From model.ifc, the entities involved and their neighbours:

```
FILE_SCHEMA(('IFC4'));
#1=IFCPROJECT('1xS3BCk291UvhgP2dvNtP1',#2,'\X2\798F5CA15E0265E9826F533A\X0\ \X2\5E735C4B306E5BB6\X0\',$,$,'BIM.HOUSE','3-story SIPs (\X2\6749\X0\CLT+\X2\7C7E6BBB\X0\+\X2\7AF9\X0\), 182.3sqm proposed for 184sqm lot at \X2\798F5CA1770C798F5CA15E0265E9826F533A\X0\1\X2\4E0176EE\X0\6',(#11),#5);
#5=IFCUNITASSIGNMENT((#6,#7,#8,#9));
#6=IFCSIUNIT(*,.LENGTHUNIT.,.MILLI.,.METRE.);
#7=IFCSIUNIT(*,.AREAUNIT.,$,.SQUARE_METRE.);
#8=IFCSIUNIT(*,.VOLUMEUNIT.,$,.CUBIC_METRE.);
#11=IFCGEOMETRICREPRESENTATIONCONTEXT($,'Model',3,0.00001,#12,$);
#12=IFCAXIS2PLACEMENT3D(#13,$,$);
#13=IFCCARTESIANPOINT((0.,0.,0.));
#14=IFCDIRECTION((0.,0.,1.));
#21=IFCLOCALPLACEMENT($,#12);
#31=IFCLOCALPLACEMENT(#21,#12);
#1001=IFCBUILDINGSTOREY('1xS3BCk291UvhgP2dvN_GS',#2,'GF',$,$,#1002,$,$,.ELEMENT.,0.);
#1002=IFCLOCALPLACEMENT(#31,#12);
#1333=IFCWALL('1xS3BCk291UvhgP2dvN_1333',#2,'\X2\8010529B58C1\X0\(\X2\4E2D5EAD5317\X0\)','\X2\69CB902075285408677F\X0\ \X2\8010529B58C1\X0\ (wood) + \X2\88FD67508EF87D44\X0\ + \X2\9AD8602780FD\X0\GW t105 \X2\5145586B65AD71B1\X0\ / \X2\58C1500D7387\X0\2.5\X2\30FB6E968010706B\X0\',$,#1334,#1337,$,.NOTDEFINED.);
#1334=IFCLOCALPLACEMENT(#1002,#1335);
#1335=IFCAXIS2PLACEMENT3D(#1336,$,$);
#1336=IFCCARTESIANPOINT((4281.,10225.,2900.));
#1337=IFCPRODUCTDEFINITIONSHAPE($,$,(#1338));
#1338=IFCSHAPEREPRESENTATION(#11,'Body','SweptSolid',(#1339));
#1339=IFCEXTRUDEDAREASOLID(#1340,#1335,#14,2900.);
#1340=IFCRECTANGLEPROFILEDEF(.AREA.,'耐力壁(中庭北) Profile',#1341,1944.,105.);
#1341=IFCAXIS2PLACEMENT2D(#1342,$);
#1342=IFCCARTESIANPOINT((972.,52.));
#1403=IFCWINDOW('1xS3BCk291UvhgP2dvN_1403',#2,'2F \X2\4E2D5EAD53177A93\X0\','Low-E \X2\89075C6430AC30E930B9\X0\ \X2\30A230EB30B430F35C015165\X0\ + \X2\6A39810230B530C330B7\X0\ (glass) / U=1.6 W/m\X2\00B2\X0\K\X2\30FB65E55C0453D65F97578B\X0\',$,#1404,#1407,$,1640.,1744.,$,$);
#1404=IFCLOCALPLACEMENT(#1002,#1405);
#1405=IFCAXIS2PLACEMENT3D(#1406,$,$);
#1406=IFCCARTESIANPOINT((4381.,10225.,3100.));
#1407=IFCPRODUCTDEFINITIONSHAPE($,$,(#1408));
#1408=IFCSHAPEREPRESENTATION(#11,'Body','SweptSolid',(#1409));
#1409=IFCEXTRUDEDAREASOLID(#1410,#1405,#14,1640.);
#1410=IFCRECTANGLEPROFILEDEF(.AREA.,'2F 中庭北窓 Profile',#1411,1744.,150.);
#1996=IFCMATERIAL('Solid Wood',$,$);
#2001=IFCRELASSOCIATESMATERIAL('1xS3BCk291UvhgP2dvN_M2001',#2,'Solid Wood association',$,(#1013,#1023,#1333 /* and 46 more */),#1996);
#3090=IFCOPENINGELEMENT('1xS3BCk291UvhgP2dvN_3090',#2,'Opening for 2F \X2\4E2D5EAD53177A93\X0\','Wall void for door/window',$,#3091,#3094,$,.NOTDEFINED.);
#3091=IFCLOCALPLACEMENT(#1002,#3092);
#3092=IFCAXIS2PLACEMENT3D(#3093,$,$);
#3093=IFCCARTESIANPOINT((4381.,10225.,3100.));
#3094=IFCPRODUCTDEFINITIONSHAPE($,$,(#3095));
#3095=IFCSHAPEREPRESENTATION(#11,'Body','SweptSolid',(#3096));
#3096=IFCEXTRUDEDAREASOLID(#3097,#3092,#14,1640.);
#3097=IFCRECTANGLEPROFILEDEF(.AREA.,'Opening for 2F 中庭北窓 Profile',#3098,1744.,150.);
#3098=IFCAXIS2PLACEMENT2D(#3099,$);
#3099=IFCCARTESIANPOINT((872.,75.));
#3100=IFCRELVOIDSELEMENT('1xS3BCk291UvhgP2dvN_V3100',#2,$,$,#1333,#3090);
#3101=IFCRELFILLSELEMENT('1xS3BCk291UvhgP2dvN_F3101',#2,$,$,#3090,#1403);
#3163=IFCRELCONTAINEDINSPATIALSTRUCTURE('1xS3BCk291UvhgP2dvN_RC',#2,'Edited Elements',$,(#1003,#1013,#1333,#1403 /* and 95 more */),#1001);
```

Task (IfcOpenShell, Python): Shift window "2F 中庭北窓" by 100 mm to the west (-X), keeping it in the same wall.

```python
import ifcopenshell
import ifcopenshell.api.geometry
import ifcopenshell.util.placement

model = ifcopenshell.open("model.ifc")

window = model.by_guid("1xS3BCk291UvhgP2dvN_1403")
opening = window.FillsVoids[0].RelatingOpeningElement
wall = opening.VoidsElements[0].RelatingBuildingElement

wall_matrix = ifcopenshell.util.placement.get_local_placement(wall.ObjectPlacement)
shift = wall_matrix[:3, 0] * -100.0
before = ifcopenshell.util.placement.get_local_placement(window.ObjectPlacement)[:3, 3].copy()

# The window is not placed relative to its opening, so move both.
for product in (opening, window):
    matrix = ifcopenshell.util.placement.get_local_placement(product.ObjectPlacement)
    matrix[:3, 3] += shift
    ifcopenshell.api.geometry.edit_object_placement(model, product=product, matrix=matrix, is_si=False)

after = ifcopenshell.util.placement.get_local_placement(window.ObjectPlacement)[:3, 3]
print("window moved by", (after - before).round(3) + 0.0)

model.write("model_rev.ifc")
```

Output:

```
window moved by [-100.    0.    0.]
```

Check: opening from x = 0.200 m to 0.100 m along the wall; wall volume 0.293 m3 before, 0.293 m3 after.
